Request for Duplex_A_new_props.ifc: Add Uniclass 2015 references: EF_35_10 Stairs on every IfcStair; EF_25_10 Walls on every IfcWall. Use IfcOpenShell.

First a look at what the model holds.

```python
import ifcopenshell

model = ifcopenshell.open("Duplex_A_new_props.ifc")
print(model.schema)
print("classifications:", [c.Name for c in model.by_type("IfcClassification")])
for ifc_class in ("IfcDoor", "IfcRoof", "IfcStair", "IfcWall", "IfcWindow"):
    print(ifc_class, len(model.by_type(ifc_class)))
```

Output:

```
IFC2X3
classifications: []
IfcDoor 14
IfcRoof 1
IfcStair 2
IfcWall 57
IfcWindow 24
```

```python
import ifcopenshell
import ifcopenshell.api.classification

model = ifcopenshell.open("Duplex_A_new_props.ifc")

# IFC2X3 requires Source and Edition and has no link from the project to the system.
system = model.create_entity("IfcClassification", Source="NBS", Edition="2015", Name="Uniclass 2015")

codes = {
    "IfcStair": ("EF_35_10", "Stairs"),
    "IfcWall": ("EF_25_10", "Walls"),
}
for ifc_class, (code, name) in codes.items():
    products = model.by_type(ifc_class)
    ifcopenshell.api.classification.add_reference(
        model, products=products, classification=system, identification=code, name=name
    )
    print(code, len(products))

model.write("Duplex_A_new_props_rev.ifc")
```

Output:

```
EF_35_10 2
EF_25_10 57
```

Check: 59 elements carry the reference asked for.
